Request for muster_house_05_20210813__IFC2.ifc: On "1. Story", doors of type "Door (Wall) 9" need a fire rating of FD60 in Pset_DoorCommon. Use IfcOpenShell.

First a look at what the model holds.

```python
import ifcopenshell
import ifcopenshell.util.element

model = ifcopenshell.open("muster_house_05_20210813__IFC2.ifc")
print(model.schema)
storey = next(s for s in model.by_type("IfcBuildingStorey") if s.Name == "1. Story")
doors = [e for e in ifcopenshell.util.element.get_decomposition(storey) if e.is_a("IfcDoor")]
seen = {}
for e in doors:
    element_type = ifcopenshell.util.element.get_type(e)
    key = (element_type.Name if element_type != e and element_type else None, ifcopenshell.util.element.get_pset(e, "Pset_DoorCommon", "FireRating"))
    seen[key] = seen.get(key, 0) + 1
for (name, value), count in sorted(seen.items(), key=str):
    print(count, "x", name, "|", value)
```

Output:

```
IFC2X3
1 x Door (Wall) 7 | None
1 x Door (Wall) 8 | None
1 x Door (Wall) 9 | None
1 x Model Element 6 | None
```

```python
import ifcopenshell
import ifcopenshell.api.pset
import ifcopenshell.util.element

model = ifcopenshell.open("muster_house_05_20210813__IFC2.ifc")

storey = next(s for s in model.by_type("IfcBuildingStorey") if s.Name == "1. Story")
doors = [e for e in ifcopenshell.util.element.get_decomposition(storey) if e.is_a("IfcDoor")]

count = 0
for e in doors:
    element_type = ifcopenshell.util.element.get_type(e)
    if element_type in (None, e) or element_type.Name != "Door (Wall) 9":
        continue
    # add_pset returns the element's existing set when there is one.
    pset = ifcopenshell.api.pset.add_pset(model, product=e, name="Pset_DoorCommon")
    ifcopenshell.api.pset.edit_pset(model, pset=pset, properties={"FireRating": "FD60"})
    count += 1

print(count, "doors updated")

model.write("muster_house_05_20210813__IFC2_edited.ifc")
```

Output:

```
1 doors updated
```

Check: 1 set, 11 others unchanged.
